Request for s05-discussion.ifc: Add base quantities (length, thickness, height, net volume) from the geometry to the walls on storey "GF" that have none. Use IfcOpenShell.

First a look at what the model holds.

```python
import ifcopenshell
import ifcopenshell.util.element
import ifcopenshell.util.unit

model = ifcopenshell.open("s05-discussion.ifc")
print(model.schema)
for unit_type in ("LENGTHUNIT", "AREAUNIT", "VOLUMEUNIT"):
    print(unit_type, ifcopenshell.util.unit.calculate_unit_scale(model, unit_type))
storey = next(s for s in model.by_type("IfcBuildingStorey") if s.Name == "GF")
walls = [e for e in ifcopenshell.util.element.get_decomposition(storey) if e.is_a("IfcWall")]
for e in sorted(walls, key=lambda e: e.id()):
    print(e.id(), e.is_a(), e.Name, list(ifcopenshell.util.element.get_psets(e, qtos_only=True)), sep=" | ")
```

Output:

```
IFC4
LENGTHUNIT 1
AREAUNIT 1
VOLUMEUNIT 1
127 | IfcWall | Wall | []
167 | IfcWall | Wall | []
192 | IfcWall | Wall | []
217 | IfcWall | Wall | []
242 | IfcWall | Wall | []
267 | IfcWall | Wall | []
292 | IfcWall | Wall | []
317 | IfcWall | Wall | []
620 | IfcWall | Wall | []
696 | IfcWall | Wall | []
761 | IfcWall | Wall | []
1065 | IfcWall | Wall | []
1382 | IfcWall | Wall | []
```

```python
import ifcopenshell
import ifcopenshell.api.pset
import ifcopenshell.geom
import ifcopenshell.util.element
import ifcopenshell.util.shape
import ifcopenshell.util.unit

model = ifcopenshell.open("s05-discussion.ifc")
unit_scale = ifcopenshell.util.unit.calculate_unit_scale(model)
volume_scale = ifcopenshell.util.unit.calculate_unit_scale(model, "VOLUMEUNIT")
settings = ifcopenshell.geom.settings()

storey = next(s for s in model.by_type("IfcBuildingStorey") if s.Name == "GF")
walls = [e for e in ifcopenshell.util.element.get_decomposition(storey) if e.is_a("IfcWall")]

for e in sorted(walls, key=lambda e: e.id()):
    if ifcopenshell.util.element.get_psets(e, qtos_only=True, should_inherit=False):
        continue
    # Geometry comes back in metres, in the element's own axes.
    shape = ifcopenshell.geom.create_shape(settings, e)
    values = {
        "Length": ifcopenshell.util.shape.get_x(shape.geometry) / unit_scale,
        "Width": ifcopenshell.util.shape.get_y(shape.geometry) / unit_scale,
        "Height": ifcopenshell.util.shape.get_z(shape.geometry) / unit_scale,
        "NetVolume": ifcopenshell.util.shape.get_volume(shape.geometry) / volume_scale,
    }
    qto = ifcopenshell.api.pset.add_qto(model, product=e, name="Qto_WallBaseQuantities")
    ifcopenshell.api.pset.edit_qto(model, qto=qto, properties=values)
    print(e.id(), {k: round(v, 3) for k, v in values.items()})

model.write("s05-discussion_rev.ifc")
```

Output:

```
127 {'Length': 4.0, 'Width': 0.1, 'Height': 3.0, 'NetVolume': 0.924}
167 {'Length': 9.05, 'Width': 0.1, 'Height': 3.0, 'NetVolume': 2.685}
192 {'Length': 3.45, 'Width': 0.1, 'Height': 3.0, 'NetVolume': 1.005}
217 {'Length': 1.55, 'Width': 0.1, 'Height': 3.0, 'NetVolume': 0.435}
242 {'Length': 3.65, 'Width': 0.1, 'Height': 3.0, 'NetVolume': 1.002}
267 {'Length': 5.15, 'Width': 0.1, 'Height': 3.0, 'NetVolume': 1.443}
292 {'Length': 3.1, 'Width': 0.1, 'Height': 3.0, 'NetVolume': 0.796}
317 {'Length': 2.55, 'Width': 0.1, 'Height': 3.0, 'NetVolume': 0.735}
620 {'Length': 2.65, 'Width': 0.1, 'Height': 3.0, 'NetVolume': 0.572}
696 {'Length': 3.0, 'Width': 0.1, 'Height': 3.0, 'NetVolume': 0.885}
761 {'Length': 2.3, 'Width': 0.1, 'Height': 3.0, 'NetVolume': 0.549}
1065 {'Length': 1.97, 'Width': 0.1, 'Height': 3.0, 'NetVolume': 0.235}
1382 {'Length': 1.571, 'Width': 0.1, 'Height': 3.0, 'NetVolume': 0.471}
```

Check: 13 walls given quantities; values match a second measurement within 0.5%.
